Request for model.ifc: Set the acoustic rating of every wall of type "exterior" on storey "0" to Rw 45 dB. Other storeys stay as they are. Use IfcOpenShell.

First a look at what the model holds.

```python
import ifcopenshell
import ifcopenshell.util.element

model = ifcopenshell.open("model.ifc")
print(model.schema)
storey = next(s for s in model.by_type("IfcBuildingStorey") if s.Name == "0")
walls = [e for e in ifcopenshell.util.element.get_decomposition(storey) if e.is_a("IfcWall")]
seen = {}
for e in walls:
    element_type = ifcopenshell.util.element.get_type(e)
    key = (element_type.Name if element_type != e and element_type else None, ifcopenshell.util.element.get_pset(e, "Pset_WallCommon", "AcousticRating"))
    seen[key] = seen.get(key, 0) + 1
for (name, value), count in sorted(seen.items(), key=str):
    print(count, "x", name, "|", value)
```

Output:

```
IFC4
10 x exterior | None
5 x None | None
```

```python
import ifcopenshell
import ifcopenshell.api.pset
import ifcopenshell.util.element

model = ifcopenshell.open("model.ifc")

storey = next(s for s in model.by_type("IfcBuildingStorey") if s.Name == "0")
walls = [e for e in ifcopenshell.util.element.get_decomposition(storey) if e.is_a("IfcWall")]

count = 0
for e in walls:
    element_type = ifcopenshell.util.element.get_type(e)
    if element_type in (None, e) or element_type.Name != "exterior":
        continue
    # add_pset returns the element's existing set when there is one.
    pset = ifcopenshell.api.pset.add_pset(model, product=e, name="Pset_WallCommon")
    ifcopenshell.api.pset.edit_pset(model, pset=pset, properties={"AcousticRating": "Rw 45 dB"})
    count += 1

print(count, "walls updated")

model.write("model-out.ifc")
```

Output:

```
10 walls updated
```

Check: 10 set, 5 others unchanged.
